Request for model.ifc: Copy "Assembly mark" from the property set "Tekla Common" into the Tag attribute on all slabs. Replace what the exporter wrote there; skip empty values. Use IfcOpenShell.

First a look at what the model holds.

```python
import ifcopenshell
import ifcopenshell.util.element

model = ifcopenshell.open("model.ifc")
print(model.schema)
slabs = model.by_type("IfcSlab")
print(len(slabs), "slabs")
for e in slabs[:8]:
    source = ifcopenshell.util.element.get_pset(e, "Tekla Common", "Assembly mark")
    target = e.Tag
    print(e.id(), repr(source), repr(target), sep=" | ")
```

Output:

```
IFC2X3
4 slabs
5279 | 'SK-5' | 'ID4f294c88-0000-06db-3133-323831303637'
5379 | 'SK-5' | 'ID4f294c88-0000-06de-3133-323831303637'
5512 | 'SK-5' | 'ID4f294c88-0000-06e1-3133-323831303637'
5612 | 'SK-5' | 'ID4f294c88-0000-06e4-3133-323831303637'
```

```python
import ifcopenshell
import ifcopenshell.util.element

model = ifcopenshell.open("model.ifc")

count = 0
for e in model.by_type("IfcSlab"):
    value = ifcopenshell.util.element.get_pset(e, "Tekla Common", "Assembly mark")
    current = e.Tag
    if not value or not value.strip() or current == value:
        continue
    e.Tag = value
    count += 1

print(count, "slabs updated")

model.write("model-out.ifc")
```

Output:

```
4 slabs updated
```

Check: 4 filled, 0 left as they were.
